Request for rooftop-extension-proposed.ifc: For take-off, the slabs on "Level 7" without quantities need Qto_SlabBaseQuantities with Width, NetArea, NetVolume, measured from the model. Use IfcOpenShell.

First a look at what the model holds.

```python
import ifcopenshell
import ifcopenshell.util.element
import ifcopenshell.util.unit

model = ifcopenshell.open("rooftop-extension-proposed.ifc")
print(model.schema)
for unit_type in ("LENGTHUNIT", "AREAUNIT", "VOLUMEUNIT"):
    print(unit_type, ifcopenshell.util.unit.calculate_unit_scale(model, unit_type))
storey = next(s for s in model.by_type("IfcBuildingStorey") if s.Name == "Level 7")
slabs = [e for e in ifcopenshell.util.element.get_decomposition(storey) if e.is_a("IfcSlab")]
for e in sorted(slabs, key=lambda e: e.id()):
    print(e.id(), e.is_a(), e.Name, list(ifcopenshell.util.element.get_psets(e, qtos_only=True)), sep=" | ")
```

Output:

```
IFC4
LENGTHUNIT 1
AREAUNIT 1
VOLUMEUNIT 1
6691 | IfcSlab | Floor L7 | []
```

```python
import ifcopenshell
import ifcopenshell.api.pset
import ifcopenshell.geom
import ifcopenshell.util.element
import ifcopenshell.util.shape
import ifcopenshell.util.unit

model = ifcopenshell.open("rooftop-extension-proposed.ifc")
unit_scale = ifcopenshell.util.unit.calculate_unit_scale(model)
area_scale = ifcopenshell.util.unit.calculate_unit_scale(model, "AREAUNIT")
volume_scale = ifcopenshell.util.unit.calculate_unit_scale(model, "VOLUMEUNIT")
settings = ifcopenshell.geom.settings()

storey = next(s for s in model.by_type("IfcBuildingStorey") if s.Name == "Level 7")
slabs = [e for e in ifcopenshell.util.element.get_decomposition(storey) if e.is_a("IfcSlab")]

for e in sorted(slabs, key=lambda e: e.id()):
    if ifcopenshell.util.element.get_psets(e, qtos_only=True, should_inherit=False):
        continue
    # Geometry comes back in metres, in the element's own axes.
    shape = ifcopenshell.geom.create_shape(settings, e)
    values = {
        "Width": ifcopenshell.util.shape.get_z(shape.geometry) / unit_scale,
        "NetArea": ifcopenshell.util.shape.get_footprint_area(shape.geometry) / area_scale,
        "NetVolume": ifcopenshell.util.shape.get_volume(shape.geometry) / volume_scale,
    }
    qto = ifcopenshell.api.pset.add_qto(model, product=e, name="Qto_SlabBaseQuantities")
    ifcopenshell.api.pset.edit_qto(model, qto=qto, properties=values)
    print(e.id(), {k: round(v, 3) for k, v in values.items()})

model.write("rooftop-extension-proposed_edited.ifc")
```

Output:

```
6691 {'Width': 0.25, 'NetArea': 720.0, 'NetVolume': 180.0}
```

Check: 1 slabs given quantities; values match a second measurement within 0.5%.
